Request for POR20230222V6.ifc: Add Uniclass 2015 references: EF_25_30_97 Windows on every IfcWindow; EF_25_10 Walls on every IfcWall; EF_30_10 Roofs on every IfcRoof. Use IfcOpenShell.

First a look at what the model holds.

```python
import ifcopenshell

model = ifcopenshell.open("POR20230222V6.ifc")
print(model.schema)
print("classifications:", [c.Name for c in model.by_type("IfcClassification")])
for ifc_class in ("IfcDoor", "IfcRoof", "IfcStair", "IfcWall", "IfcWindow"):
    print(ifc_class, len(model.by_type(ifc_class)))
```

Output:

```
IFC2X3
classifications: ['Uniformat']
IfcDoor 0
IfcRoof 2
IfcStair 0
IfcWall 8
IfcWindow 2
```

```python
import ifcopenshell
import ifcopenshell.api.classification

model = ifcopenshell.open("POR20230222V6.ifc")

# IFC2X3 requires Source and Edition and has no link from the project to the system.
system = model.create_entity("IfcClassification", Source="NBS", Edition="2015", Name="Uniclass 2015")

codes = {
    "IfcWindow": ("EF_25_30_97", "Windows"),
    "IfcWall": ("EF_25_10", "Walls"),
    "IfcRoof": ("EF_30_10", "Roofs"),
}
for ifc_class, (code, name) in codes.items():
    products = model.by_type(ifc_class)
    ifcopenshell.api.classification.add_reference(
        model, products=products, classification=system, identification=code, name=name
    )
    print(code, len(products))

model.write("POR20230222V6_v2.ifc")
```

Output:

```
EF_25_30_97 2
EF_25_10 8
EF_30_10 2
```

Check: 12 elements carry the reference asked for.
